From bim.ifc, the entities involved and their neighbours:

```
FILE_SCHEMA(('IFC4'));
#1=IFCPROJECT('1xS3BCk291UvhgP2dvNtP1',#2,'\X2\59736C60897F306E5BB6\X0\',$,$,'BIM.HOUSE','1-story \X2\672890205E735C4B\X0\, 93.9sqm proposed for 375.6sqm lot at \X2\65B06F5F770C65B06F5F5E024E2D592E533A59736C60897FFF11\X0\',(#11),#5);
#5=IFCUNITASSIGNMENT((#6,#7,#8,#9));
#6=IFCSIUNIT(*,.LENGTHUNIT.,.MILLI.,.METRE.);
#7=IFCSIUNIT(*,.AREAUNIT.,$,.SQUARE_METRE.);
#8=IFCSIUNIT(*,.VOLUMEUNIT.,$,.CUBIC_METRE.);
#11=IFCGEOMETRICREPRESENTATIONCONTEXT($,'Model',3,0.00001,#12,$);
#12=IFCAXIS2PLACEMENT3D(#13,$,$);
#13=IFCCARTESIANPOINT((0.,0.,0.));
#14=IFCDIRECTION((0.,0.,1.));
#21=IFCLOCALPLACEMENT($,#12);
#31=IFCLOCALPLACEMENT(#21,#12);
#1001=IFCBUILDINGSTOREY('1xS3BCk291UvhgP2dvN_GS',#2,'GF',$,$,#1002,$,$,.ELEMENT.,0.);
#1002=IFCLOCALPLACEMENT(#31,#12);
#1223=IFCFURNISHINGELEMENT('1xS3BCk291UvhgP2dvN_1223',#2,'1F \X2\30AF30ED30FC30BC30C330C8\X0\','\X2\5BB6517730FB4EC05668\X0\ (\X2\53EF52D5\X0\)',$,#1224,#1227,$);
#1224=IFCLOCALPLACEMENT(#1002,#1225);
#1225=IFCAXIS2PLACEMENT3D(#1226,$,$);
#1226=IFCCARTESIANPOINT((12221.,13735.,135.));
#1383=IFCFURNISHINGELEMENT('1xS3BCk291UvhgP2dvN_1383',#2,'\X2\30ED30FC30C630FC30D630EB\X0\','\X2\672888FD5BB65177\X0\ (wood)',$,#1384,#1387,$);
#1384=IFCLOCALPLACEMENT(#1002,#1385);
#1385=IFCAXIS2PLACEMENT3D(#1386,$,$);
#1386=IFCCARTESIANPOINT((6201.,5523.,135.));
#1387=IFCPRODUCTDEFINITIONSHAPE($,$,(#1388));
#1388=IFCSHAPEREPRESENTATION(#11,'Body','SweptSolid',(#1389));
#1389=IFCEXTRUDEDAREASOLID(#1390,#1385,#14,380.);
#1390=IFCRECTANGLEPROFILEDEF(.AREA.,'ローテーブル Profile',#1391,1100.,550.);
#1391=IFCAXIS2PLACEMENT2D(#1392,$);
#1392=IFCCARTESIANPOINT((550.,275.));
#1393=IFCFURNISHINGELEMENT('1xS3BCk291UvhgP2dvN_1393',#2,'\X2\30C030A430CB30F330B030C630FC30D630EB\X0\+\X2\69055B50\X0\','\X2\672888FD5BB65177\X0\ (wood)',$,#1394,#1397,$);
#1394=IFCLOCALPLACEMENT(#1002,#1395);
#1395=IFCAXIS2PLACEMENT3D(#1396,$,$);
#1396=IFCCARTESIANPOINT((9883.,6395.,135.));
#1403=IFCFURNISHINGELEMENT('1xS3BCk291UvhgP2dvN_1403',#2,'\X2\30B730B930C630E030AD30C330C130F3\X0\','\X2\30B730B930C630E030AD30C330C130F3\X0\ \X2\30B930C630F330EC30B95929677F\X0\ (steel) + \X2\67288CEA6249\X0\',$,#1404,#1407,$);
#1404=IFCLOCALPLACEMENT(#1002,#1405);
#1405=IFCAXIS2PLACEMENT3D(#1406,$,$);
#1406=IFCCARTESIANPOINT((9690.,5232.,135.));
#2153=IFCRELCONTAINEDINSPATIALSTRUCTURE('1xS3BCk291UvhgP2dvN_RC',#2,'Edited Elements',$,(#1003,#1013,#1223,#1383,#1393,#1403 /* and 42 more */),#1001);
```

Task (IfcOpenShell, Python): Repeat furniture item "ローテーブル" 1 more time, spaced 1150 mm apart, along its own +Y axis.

```python
import ifcopenshell
import ifcopenshell.api.geometry
import ifcopenshell.api.root
import ifcopenshell.util.element
import ifcopenshell.util.placement

model = ifcopenshell.open("bim.ifc")


def reuse_history(source, copy):
    """copy_class also copies each property set's owner history, people and application; keep the originals."""
    for rel in copy.IsDefinedBy:
        if rel.is_a("IfcRelDefinesByProperties") and (history := rel.RelatingPropertyDefinition.OwnerHistory):
            rel.RelatingPropertyDefinition.OwnerHistory = source.OwnerHistory
            ifcopenshell.util.element.remove_deep2(model, history)


source = model.by_guid("1xS3BCk291UvhgP2dvN_1383")
base = ifcopenshell.util.placement.get_local_placement(source.ObjectPlacement)
step = base[:3, 1] * 1150.0

for i in range(1, 2):
    copy = ifcopenshell.api.root.copy_class(model, product=source)
    copy.Representation = ifcopenshell.util.element.copy_deep(
        model, source.Representation, exclude=["IfcGeometricRepresentationContext", "IfcRepresentationMap"]
    )
    reuse_history(source, copy)
    matrix = base.copy()
    matrix[:3, 3] += i * step
    print("added at", matrix[:3, 3].round(3) + 0.0)
    ifcopenshell.api.geometry.edit_object_placement(model, product=copy, matrix=matrix, is_si=False)

model.write("bim_updated.ifc")
```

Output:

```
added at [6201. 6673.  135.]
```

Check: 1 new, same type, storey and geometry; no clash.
